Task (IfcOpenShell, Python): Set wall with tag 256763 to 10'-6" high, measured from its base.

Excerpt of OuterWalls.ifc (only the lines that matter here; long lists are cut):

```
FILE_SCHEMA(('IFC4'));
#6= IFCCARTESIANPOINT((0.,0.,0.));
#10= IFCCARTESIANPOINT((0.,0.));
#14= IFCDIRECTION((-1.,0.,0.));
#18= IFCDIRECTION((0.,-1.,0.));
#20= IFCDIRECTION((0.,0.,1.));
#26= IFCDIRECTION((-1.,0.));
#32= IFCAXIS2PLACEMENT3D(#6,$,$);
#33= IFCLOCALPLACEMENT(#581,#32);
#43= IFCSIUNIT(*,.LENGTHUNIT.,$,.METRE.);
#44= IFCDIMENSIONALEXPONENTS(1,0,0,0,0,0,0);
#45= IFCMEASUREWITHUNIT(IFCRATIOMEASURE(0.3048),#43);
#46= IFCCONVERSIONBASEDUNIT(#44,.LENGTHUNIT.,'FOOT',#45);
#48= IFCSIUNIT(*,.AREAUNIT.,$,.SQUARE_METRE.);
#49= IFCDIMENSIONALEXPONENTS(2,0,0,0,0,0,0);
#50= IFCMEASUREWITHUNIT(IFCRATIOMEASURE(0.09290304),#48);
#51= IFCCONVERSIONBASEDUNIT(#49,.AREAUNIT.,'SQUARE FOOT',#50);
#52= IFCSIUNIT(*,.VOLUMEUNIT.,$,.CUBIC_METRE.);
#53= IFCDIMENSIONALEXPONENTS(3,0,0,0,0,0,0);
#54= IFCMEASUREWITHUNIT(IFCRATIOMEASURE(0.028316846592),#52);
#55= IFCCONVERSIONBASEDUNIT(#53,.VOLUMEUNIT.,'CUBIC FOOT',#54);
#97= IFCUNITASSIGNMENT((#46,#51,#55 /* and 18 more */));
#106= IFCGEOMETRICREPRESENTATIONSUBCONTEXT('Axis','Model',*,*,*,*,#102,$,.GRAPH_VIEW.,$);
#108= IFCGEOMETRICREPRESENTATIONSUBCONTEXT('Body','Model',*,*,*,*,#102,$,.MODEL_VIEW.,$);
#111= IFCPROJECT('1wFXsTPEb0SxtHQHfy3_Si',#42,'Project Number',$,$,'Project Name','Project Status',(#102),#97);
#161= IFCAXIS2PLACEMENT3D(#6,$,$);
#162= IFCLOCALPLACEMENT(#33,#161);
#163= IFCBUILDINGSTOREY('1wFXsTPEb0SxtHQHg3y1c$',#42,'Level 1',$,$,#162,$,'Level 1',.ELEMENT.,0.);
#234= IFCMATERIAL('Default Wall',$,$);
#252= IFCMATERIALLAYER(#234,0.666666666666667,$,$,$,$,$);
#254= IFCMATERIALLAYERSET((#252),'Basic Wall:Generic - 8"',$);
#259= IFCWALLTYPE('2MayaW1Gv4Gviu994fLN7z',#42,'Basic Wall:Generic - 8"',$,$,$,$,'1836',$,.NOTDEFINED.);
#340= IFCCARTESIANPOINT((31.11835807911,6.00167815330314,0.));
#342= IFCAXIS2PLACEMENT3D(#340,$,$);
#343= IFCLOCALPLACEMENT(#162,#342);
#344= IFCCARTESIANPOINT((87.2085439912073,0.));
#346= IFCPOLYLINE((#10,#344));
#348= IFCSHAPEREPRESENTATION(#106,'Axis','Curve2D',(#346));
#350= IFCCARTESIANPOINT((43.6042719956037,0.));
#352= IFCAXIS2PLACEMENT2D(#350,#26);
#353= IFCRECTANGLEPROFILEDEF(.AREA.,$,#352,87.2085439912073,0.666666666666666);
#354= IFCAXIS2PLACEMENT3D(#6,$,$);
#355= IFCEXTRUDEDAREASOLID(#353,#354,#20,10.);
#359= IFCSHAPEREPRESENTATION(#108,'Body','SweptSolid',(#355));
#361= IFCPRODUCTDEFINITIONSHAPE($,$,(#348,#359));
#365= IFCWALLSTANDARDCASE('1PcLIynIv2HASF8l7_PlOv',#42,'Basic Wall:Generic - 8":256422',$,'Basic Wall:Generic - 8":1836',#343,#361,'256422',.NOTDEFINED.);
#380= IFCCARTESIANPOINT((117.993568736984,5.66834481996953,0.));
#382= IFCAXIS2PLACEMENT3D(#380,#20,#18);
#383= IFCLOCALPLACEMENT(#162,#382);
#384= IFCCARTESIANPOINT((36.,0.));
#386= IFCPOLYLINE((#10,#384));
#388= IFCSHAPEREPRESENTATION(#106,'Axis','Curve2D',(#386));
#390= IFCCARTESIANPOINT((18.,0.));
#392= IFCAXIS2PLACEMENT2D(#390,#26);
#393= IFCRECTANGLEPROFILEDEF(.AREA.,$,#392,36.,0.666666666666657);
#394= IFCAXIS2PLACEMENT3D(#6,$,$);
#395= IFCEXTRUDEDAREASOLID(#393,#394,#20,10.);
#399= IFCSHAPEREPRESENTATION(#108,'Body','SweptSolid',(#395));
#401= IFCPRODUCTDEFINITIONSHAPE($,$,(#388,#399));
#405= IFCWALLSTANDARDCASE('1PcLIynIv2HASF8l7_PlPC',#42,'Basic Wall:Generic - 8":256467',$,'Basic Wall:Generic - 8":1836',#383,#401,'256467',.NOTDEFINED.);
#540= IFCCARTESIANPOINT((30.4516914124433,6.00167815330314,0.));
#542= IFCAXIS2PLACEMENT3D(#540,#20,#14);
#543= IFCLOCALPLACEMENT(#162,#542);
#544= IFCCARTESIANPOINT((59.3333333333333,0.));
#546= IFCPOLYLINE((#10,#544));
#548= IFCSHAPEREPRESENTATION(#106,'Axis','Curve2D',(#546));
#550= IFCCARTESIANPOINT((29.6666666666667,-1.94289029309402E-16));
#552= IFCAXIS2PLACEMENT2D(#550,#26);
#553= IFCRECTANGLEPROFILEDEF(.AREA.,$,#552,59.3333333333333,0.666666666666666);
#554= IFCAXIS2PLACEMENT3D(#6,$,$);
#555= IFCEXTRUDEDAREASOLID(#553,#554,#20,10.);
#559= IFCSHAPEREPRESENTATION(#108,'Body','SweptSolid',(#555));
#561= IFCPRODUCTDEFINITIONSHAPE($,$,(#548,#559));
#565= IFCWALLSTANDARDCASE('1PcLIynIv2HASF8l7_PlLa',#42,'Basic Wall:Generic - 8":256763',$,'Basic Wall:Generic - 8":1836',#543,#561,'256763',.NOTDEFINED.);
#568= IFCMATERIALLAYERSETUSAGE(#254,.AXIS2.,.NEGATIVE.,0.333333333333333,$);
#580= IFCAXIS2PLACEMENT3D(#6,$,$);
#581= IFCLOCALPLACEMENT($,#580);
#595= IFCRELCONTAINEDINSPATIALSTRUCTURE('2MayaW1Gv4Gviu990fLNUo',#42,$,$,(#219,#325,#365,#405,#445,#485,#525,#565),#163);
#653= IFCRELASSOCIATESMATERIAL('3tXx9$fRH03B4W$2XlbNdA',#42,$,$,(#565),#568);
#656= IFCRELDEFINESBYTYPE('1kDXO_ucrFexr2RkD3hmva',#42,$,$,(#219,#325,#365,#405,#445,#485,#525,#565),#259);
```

```python
import ifcopenshell
import ifcopenshell.geom
import ifcopenshell.util.representation
import ifcopenshell.util.shape
import ifcopenshell.util.unit

model = ifcopenshell.open("OuterWalls.ifc")
unit_scale = ifcopenshell.util.unit.calculate_unit_scale(model)
settings = ifcopenshell.geom.settings()


def volume(element):
    """Net volume in cubic metres, openings subtracted."""
    shape = ifcopenshell.geom.create_shape(settings, element)
    return ifcopenshell.util.shape.get_volume(shape.geometry)


wall = model.by_guid("1PcLIynIv2HASF8l7_PlLa")
before = volume(wall)

body = ifcopenshell.util.representation.get_representation(wall, "Model", "Body")
solid = body.Items[0]
old_height = solid.Depth
solid.Depth = 126 * 0.0254 / unit_scale
after = volume(wall)

print(f"height {old_height:g} -> {solid.Depth:g}, volume {before:.3f} -> {after:.3f} m3")

model.write("OuterWalls_rev.ifc")
```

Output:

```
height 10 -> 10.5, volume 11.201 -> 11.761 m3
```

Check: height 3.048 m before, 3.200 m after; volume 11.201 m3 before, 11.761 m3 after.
